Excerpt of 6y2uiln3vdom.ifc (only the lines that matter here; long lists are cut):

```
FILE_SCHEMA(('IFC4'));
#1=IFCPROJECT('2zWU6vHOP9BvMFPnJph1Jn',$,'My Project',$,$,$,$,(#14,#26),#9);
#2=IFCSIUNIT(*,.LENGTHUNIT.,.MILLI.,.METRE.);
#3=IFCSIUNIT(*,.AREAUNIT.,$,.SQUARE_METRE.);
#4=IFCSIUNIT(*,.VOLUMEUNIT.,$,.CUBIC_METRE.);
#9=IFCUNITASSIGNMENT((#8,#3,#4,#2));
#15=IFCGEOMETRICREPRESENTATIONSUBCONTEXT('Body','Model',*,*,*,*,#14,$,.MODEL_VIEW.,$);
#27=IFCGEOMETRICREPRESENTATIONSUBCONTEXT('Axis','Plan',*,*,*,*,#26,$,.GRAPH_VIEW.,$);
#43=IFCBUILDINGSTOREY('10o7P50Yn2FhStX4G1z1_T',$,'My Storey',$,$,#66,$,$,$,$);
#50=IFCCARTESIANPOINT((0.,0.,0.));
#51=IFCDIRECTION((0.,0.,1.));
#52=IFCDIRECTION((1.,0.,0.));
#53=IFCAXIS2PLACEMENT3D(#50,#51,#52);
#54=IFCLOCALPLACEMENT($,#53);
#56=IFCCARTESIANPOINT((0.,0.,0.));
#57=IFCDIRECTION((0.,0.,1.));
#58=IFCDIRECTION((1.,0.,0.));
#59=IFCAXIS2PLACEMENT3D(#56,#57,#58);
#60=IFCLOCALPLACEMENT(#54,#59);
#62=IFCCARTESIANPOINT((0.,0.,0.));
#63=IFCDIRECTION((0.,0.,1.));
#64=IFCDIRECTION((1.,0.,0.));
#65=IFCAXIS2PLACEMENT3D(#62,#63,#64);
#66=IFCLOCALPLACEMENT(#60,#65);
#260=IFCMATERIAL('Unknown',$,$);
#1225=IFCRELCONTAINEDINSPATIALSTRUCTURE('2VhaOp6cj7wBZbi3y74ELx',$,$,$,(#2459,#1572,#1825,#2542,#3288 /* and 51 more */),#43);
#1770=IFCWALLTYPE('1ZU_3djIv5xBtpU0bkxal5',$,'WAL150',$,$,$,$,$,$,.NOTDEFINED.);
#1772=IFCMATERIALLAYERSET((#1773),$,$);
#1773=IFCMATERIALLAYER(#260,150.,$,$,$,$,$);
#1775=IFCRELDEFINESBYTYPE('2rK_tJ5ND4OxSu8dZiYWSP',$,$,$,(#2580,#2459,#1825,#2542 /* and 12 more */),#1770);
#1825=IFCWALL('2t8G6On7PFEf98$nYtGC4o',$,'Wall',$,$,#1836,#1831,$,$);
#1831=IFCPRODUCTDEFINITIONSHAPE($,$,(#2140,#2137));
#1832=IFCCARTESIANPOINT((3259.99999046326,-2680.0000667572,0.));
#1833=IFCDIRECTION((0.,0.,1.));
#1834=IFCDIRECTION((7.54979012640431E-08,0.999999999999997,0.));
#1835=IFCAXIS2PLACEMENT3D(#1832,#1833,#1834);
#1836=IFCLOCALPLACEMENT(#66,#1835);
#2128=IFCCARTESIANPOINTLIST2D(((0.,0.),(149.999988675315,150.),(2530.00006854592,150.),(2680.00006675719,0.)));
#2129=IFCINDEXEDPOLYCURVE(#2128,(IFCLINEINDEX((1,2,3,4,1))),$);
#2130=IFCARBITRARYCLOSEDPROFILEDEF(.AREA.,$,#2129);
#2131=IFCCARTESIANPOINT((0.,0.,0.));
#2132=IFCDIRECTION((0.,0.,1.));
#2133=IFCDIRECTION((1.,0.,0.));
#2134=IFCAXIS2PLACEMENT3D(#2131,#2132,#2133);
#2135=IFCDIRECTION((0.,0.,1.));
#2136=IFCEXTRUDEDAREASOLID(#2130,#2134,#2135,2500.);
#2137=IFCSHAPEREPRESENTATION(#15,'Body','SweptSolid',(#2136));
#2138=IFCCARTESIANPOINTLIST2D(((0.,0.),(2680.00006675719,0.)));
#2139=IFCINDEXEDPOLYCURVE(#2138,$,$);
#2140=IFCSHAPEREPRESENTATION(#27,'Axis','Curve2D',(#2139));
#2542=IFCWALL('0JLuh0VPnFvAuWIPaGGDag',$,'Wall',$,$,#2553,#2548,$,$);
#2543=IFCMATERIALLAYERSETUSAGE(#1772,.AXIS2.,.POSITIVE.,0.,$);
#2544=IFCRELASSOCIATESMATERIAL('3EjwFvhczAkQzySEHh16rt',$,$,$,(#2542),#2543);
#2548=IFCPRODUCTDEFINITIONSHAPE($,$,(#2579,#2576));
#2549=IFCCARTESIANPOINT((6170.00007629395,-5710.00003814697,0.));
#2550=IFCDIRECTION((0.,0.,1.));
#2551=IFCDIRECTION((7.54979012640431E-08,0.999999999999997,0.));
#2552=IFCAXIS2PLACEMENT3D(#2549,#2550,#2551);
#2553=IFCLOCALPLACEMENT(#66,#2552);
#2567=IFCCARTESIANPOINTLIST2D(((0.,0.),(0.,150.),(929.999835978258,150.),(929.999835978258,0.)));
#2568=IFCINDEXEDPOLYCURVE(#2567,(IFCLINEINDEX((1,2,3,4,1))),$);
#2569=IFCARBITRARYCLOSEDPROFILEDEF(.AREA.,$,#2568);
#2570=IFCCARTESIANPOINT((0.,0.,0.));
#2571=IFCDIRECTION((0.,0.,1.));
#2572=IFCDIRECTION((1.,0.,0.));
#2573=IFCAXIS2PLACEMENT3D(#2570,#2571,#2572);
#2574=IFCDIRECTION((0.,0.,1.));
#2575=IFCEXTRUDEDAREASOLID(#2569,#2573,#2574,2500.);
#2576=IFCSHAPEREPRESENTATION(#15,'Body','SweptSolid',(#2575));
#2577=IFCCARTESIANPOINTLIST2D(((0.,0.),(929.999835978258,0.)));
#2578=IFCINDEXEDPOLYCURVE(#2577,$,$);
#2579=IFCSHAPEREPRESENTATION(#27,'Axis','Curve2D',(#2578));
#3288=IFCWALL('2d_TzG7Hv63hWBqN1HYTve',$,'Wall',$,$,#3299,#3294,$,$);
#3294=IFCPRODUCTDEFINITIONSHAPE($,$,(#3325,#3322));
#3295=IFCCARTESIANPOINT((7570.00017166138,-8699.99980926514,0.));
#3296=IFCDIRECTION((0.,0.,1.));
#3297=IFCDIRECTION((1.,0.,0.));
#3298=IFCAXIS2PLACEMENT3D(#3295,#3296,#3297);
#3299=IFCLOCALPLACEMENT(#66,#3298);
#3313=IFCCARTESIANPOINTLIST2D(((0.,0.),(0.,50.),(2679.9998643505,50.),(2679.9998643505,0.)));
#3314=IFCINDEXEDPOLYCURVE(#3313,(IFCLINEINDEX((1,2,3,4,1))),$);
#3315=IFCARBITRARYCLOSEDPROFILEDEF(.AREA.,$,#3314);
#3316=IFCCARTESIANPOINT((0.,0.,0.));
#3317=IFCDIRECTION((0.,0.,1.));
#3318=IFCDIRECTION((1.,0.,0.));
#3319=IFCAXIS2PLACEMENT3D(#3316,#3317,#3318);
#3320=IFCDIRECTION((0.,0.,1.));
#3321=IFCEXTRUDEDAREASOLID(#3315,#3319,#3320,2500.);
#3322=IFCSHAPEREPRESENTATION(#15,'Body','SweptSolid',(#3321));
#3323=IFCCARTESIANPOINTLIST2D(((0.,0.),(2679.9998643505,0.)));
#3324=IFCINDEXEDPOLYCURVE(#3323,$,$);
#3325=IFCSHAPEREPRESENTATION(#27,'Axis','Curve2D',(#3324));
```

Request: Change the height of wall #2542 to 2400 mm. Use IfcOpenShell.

```python
import ifcopenshell
import ifcopenshell.geom
import ifcopenshell.util.representation
import ifcopenshell.util.shape

model = ifcopenshell.open("6y2uiln3vdom.ifc")
settings = ifcopenshell.geom.settings()


def volume(element):
    """Net volume in cubic metres, openings subtracted."""
    shape = ifcopenshell.geom.create_shape(settings, element)
    return ifcopenshell.util.shape.get_volume(shape.geometry)


wall = model.by_guid("0JLuh0VPnFvAuWIPaGGDag")
before = volume(wall)

body = ifcopenshell.util.representation.get_representation(wall, "Model", "Body")
solid = body.Items[0]
old_height = solid.Depth
solid.Depth = 2400.0
after = volume(wall)

print(f"height {old_height:g} -> {solid.Depth:g}, volume {before:.3f} -> {after:.3f} m3")

model.write("6y2uiln3vdom_edited.ifc")
```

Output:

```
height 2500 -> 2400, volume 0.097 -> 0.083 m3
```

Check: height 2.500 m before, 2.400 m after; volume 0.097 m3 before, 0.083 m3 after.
